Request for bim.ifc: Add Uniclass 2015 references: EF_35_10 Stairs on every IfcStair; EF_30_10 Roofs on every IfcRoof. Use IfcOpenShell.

First a look at what the model holds.

```python
import ifcopenshell

model = ifcopenshell.open("bim.ifc")
print(model.schema)
print("classifications:", [c.Name for c in model.by_type("IfcClassification")])
for ifc_class in ("IfcDoor", "IfcRoof", "IfcStair", "IfcWall", "IfcWindow"):
    print(ifc_class, len(model.by_type(ifc_class)))
```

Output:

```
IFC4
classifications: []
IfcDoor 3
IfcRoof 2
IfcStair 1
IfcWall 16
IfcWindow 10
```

```python
import ifcopenshell
import ifcopenshell.api.classification

model = ifcopenshell.open("bim.ifc")

system = ifcopenshell.api.classification.add_classification(model, classification="Uniclass 2015")

codes = {
    "IfcStair": ("EF_35_10", "Stairs"),
    "IfcRoof": ("EF_30_10", "Roofs"),
}
for ifc_class, (code, name) in codes.items():
    products = model.by_type(ifc_class)
    ifcopenshell.api.classification.add_reference(
        model, products=products, classification=system, identification=code, name=name
    )
    print(code, len(products))

model.write("bim_v2.ifc")
```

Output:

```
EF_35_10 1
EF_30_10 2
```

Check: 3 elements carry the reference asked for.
